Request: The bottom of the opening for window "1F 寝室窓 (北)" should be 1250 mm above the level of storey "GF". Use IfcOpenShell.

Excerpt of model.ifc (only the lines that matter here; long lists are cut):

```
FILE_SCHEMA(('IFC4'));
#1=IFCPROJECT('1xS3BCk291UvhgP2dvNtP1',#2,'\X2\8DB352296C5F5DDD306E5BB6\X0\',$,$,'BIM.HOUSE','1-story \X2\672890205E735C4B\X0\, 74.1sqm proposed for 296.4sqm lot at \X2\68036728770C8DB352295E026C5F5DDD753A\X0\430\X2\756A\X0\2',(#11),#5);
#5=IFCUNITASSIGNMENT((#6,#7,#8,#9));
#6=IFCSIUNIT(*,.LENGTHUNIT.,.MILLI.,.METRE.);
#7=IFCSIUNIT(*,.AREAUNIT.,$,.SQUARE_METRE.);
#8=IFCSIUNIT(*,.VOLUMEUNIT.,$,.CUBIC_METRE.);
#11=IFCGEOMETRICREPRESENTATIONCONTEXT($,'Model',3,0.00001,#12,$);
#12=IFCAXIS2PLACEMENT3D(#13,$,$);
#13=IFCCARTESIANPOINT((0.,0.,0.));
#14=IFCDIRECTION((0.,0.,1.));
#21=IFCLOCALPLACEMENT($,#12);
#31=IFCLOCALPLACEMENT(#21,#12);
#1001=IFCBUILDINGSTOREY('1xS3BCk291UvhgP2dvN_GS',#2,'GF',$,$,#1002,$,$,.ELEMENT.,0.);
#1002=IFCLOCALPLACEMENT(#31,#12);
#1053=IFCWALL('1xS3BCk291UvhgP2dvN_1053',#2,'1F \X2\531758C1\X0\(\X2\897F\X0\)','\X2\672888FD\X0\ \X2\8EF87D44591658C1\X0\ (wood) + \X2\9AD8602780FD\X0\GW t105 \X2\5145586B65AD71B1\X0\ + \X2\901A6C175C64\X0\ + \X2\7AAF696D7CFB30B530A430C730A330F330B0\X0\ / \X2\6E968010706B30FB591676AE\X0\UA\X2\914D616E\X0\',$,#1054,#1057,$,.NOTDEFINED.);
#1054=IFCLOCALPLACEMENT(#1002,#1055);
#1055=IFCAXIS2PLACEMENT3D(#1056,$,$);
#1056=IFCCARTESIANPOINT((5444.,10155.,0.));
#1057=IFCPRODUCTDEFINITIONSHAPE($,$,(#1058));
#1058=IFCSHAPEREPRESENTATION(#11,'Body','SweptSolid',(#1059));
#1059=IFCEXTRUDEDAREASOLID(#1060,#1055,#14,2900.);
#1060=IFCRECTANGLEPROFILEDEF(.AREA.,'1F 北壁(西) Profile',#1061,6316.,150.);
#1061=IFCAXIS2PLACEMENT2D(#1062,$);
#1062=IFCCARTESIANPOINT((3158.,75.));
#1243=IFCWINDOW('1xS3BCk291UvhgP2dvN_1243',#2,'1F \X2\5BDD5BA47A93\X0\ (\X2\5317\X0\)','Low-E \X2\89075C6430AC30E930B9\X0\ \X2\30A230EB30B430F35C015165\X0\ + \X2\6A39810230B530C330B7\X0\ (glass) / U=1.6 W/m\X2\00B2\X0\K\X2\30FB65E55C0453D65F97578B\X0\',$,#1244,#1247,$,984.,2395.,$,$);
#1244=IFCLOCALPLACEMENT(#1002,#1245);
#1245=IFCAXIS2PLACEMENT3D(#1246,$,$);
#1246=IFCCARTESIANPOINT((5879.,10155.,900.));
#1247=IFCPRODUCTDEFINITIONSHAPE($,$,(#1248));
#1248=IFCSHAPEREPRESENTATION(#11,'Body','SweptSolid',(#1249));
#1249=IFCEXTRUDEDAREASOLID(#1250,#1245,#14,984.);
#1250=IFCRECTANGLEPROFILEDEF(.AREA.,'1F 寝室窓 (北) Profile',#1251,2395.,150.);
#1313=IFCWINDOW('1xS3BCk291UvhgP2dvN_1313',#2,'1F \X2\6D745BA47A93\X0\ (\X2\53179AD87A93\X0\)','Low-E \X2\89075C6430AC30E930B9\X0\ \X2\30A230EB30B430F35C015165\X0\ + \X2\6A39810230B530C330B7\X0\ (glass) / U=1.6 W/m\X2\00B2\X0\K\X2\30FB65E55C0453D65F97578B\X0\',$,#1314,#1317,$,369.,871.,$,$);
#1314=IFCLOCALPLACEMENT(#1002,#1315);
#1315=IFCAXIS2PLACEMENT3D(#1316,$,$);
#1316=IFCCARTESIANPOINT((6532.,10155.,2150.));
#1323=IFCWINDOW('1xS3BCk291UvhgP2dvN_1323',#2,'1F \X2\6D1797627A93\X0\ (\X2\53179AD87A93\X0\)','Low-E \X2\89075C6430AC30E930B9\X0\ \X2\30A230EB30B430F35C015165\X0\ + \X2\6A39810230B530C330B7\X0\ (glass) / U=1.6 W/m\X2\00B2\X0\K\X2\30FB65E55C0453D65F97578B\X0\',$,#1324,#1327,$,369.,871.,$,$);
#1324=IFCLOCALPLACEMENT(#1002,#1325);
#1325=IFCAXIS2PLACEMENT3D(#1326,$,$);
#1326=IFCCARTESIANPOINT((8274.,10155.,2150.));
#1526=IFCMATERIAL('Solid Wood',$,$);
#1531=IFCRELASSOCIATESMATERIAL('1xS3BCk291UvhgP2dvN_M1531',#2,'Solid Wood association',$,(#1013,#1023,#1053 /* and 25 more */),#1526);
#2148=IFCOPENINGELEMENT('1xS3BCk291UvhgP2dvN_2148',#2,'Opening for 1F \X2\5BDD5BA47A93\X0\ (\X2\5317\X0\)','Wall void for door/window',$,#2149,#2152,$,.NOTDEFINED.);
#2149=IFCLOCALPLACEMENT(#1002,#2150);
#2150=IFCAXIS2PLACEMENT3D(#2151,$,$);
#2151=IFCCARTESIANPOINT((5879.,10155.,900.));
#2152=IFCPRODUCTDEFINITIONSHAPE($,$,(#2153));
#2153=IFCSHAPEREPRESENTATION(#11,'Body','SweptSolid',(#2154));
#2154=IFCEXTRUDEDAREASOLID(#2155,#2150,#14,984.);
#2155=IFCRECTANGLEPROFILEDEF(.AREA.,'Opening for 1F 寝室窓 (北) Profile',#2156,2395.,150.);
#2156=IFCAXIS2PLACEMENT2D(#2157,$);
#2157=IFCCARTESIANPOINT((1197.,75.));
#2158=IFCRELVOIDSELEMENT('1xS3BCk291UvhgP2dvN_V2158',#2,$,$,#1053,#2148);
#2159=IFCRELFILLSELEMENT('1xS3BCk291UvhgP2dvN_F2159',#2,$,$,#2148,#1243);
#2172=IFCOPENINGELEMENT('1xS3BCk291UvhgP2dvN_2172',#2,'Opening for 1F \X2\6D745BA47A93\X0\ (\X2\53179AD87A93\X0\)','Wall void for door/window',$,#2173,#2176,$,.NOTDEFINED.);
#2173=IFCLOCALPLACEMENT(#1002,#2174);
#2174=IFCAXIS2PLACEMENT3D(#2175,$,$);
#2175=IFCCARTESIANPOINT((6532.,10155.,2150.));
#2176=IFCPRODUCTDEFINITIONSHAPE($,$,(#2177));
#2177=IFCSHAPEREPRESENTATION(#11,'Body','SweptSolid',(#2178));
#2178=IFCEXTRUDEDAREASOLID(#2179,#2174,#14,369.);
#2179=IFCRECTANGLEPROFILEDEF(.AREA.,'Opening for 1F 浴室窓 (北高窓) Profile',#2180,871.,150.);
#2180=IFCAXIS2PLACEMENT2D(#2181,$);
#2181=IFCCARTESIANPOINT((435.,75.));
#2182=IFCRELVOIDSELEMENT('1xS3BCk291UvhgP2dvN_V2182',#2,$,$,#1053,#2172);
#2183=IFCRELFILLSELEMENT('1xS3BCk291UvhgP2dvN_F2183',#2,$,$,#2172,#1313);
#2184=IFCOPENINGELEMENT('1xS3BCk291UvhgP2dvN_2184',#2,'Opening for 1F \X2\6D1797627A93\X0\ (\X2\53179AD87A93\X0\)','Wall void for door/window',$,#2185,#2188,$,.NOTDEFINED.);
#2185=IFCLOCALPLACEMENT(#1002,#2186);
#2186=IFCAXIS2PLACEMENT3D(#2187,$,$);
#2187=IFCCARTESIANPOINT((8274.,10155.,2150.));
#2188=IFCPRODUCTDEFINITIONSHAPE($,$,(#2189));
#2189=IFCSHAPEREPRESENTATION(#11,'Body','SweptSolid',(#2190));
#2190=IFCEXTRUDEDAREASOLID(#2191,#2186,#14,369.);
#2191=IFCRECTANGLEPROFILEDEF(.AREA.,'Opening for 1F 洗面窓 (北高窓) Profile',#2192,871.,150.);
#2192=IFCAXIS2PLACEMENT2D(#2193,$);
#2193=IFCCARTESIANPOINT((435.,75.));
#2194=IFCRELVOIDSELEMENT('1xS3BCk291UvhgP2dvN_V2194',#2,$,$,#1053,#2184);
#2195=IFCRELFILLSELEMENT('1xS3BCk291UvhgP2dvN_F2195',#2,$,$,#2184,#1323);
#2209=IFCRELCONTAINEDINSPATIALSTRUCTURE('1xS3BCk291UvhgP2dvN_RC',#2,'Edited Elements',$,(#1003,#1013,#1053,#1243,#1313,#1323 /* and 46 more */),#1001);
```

```python
import numpy as np
import ifcopenshell
import ifcopenshell.api.geometry
import ifcopenshell.geom
import ifcopenshell.util.element
import ifcopenshell.util.placement
import ifcopenshell.util.shape
import ifcopenshell.util.unit

model = ifcopenshell.open("model.ifc")
unit_scale = ifcopenshell.util.unit.calculate_unit_scale(model)

window = model.by_guid("1xS3BCk291UvhgP2dvN_1243")
opening = window.FillsVoids[0].RelatingOpeningElement
storey = ifcopenshell.util.element.get_container(window, ifc_class="IfcBuildingStorey")
level = ifcopenshell.util.placement.get_local_placement(storey.ObjectPlacement)[2, 3]

# The opening's origin need not be at the sill, so measure its lowest point.
shape = ifcopenshell.geom.create_shape(ifcopenshell.geom.settings(), opening)
bottom = ifcopenshell.util.shape.get_shape_bottom_elevation(shape, shape.geometry) / unit_scale
dz = level + 1250.0 - bottom

shift = np.array([0.0, 0.0, dz])
# The window is not placed relative to its opening, so move both.
for product in (opening, window):
    matrix = ifcopenshell.util.placement.get_local_placement(product.ObjectPlacement)
    matrix[:3, 3] += shift
    ifcopenshell.api.geometry.edit_object_placement(model, product=product, matrix=matrix, is_si=False)

print(f"moved by {dz * unit_scale:+.3f} m")

model.write("model_rev.ifc")
```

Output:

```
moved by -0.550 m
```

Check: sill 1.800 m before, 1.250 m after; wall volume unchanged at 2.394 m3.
